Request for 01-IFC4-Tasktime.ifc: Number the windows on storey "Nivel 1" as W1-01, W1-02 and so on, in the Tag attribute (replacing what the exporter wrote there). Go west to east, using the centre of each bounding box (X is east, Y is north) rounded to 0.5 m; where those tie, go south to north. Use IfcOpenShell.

First a look at what the model holds.

```python
import ifcopenshell
import ifcopenshell.util.element
import ifcopenshell.util.placement

model = ifcopenshell.open("01-IFC4-Tasktime.ifc")
print(model.schema)
storey = next(s for s in model.by_type("IfcBuildingStorey") if s.Name == "Nivel 1")
windows = [e for e in ifcopenshell.util.element.get_decomposition(storey) if e.is_a("IfcWindow")]
for e in sorted(windows, key=lambda e: e.id()):
    origin = ifcopenshell.util.placement.get_local_placement(e.ObjectPlacement)[:3, 3]
    print(e.id(), e.Tag, e.Name, origin.round(2) + 0.0, sep=" | ")
```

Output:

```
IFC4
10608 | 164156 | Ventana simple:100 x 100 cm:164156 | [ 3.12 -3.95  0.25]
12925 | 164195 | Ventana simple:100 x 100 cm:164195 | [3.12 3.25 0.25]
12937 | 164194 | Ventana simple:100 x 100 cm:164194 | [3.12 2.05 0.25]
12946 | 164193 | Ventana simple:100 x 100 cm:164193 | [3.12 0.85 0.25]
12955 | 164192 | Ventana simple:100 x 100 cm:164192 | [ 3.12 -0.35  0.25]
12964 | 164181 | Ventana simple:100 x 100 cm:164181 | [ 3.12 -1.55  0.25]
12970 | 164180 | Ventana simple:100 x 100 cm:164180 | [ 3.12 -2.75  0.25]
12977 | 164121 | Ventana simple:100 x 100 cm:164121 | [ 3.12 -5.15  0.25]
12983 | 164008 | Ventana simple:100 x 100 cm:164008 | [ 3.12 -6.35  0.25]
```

```python
import ifcopenshell
import ifcopenshell.geom
import ifcopenshell.util.element
import ifcopenshell.util.shape

model = ifcopenshell.open("01-IFC4-Tasktime.ifc")
settings = ifcopenshell.geom.settings()
settings.set("use-world-coords", True)


def centre(element):
    shape = ifcopenshell.geom.create_shape(settings, element)
    return ifcopenshell.util.shape.get_bbox_centroid(shape.geometry)


storey = next(s for s in model.by_type("IfcBuildingStorey") if s.Name == "Nivel 1")
windows = [e for e in ifcopenshell.util.element.get_decomposition(storey) if e.is_a("IfcWindow")]

# Insertion points can sit at a corner or the storey origin, so sort by the geometry (in metres).
centres = {e: centre(e) for e in windows}
windows.sort(key=lambda e: (round(centres[e][0] / 0.5), centres[e][1]))

for i, e in enumerate(windows, start=1):
    number = f"W1-{i:02d}"
    e.Tag = number
    print(e.id(), number)

model.write("01-IFC4-Tasktime_updated.ifc")
```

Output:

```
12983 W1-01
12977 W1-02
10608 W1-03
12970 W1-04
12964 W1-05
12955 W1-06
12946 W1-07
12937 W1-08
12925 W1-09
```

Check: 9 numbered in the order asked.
